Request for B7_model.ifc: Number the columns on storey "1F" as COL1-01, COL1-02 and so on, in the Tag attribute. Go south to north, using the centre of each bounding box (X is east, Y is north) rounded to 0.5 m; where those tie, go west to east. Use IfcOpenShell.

First a look at what the model holds.

```python
import ifcopenshell
import ifcopenshell.util.element
import ifcopenshell.util.placement

model = ifcopenshell.open("B7_model.ifc")
print(model.schema)
storey = next(s for s in model.by_type("IfcBuildingStorey") if s.Name == "1F")
columns = [e for e in ifcopenshell.util.element.get_decomposition(storey) if e.is_a("IfcColumn")]
for e in sorted(columns, key=lambda e: e.id()):
    origin = ifcopenshell.util.placement.get_local_placement(e.ObjectPlacement)[:3, 3]
    print(e.id(), e.Tag, e.Name, origin.round(2) + 0.0, sep=" | ")
```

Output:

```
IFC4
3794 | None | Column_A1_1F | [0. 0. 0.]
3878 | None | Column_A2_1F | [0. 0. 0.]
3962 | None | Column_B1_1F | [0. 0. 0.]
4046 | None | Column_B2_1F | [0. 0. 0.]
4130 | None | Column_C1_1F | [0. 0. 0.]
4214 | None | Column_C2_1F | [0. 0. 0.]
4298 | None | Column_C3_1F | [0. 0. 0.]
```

```python
import ifcopenshell
import ifcopenshell.geom
import ifcopenshell.util.element
import ifcopenshell.util.shape

model = ifcopenshell.open("B7_model.ifc")
settings = ifcopenshell.geom.settings()
settings.set("use-world-coords", True)


def centre(element):
    shape = ifcopenshell.geom.create_shape(settings, element)
    return ifcopenshell.util.shape.get_bbox_centroid(shape.geometry)


storey = next(s for s in model.by_type("IfcBuildingStorey") if s.Name == "1F")
columns = [e for e in ifcopenshell.util.element.get_decomposition(storey) if e.is_a("IfcColumn")]

# Insertion points can sit at a corner or the storey origin, so sort by the geometry (in metres).
centres = {e: centre(e) for e in columns}
columns.sort(key=lambda e: (round(centres[e][1] / 0.5), centres[e][0]))

for i, e in enumerate(columns, start=1):
    number = f"COL1-{i:02d}"
    e.Tag = number
    print(e.id(), number)

model.write("B7_model_rev.ifc")
```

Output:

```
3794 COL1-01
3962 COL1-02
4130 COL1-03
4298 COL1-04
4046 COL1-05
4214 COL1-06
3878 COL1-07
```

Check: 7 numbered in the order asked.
